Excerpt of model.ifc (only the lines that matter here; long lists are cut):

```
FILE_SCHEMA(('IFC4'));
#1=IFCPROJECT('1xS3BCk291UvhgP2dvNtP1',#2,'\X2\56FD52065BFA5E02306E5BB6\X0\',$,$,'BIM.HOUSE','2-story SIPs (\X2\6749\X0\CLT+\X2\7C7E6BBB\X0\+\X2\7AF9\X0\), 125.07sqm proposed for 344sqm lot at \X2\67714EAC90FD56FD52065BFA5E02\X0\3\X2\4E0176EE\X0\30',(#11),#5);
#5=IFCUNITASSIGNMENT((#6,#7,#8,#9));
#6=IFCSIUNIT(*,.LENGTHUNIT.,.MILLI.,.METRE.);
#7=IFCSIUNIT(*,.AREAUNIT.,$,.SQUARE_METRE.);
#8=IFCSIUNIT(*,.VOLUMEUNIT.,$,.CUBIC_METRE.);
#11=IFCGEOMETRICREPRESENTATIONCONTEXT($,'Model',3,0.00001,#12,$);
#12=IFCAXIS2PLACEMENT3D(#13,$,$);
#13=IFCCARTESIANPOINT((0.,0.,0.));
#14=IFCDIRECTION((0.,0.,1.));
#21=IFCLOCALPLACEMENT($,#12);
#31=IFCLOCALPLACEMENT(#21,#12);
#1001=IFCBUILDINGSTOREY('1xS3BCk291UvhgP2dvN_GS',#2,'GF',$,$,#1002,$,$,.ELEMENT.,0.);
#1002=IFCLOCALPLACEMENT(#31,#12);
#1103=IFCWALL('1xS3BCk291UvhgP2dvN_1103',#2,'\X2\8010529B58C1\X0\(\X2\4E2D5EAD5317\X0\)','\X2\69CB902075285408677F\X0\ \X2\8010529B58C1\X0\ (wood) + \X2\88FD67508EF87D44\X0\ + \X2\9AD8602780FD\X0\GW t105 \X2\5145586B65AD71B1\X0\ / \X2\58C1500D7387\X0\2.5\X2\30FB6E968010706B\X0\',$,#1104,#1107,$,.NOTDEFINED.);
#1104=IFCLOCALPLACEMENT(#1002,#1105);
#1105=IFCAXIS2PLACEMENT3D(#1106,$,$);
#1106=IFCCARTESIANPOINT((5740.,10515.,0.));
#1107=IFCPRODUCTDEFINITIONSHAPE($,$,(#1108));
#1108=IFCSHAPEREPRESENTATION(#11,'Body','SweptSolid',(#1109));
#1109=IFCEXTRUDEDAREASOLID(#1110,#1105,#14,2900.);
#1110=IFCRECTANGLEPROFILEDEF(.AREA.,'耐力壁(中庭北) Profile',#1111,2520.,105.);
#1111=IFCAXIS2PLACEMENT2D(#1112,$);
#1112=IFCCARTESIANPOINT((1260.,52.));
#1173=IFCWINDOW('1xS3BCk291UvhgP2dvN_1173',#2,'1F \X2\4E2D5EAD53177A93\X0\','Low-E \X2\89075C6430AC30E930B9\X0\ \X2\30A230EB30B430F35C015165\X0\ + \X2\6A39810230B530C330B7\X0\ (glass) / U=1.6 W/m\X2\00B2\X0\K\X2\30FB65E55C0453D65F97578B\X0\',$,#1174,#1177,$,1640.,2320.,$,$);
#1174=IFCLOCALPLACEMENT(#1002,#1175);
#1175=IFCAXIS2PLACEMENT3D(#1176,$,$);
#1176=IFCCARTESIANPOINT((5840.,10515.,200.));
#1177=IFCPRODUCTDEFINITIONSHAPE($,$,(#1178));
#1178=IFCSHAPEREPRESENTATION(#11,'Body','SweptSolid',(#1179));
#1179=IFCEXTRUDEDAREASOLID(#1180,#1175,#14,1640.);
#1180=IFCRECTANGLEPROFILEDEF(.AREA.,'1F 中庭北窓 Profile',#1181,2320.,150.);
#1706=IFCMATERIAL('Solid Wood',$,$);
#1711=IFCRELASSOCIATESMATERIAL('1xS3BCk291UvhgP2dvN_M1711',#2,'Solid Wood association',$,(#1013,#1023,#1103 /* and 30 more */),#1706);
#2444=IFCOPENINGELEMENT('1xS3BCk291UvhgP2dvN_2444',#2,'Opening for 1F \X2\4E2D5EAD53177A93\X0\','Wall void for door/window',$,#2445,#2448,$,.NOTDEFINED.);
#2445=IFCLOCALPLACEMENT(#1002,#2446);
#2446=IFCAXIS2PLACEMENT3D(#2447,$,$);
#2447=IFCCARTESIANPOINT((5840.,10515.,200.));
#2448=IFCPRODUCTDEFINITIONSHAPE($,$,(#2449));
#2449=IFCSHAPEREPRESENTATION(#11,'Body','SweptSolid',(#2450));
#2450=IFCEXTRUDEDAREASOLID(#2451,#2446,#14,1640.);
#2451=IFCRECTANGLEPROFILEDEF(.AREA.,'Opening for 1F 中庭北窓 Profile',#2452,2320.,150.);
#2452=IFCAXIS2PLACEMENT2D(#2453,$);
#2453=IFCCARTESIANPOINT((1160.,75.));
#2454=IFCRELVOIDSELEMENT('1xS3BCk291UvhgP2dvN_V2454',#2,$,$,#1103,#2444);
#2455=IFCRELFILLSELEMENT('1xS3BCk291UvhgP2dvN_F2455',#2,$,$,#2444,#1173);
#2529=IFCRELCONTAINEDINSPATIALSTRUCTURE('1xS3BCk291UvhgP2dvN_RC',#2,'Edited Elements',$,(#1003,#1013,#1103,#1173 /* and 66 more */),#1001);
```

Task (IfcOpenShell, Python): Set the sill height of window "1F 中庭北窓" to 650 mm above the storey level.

```python
import numpy as np
import ifcopenshell
import ifcopenshell.api.geometry
import ifcopenshell.geom
import ifcopenshell.util.element
import ifcopenshell.util.placement
import ifcopenshell.util.shape
import ifcopenshell.util.unit

model = ifcopenshell.open("model.ifc")
unit_scale = ifcopenshell.util.unit.calculate_unit_scale(model)

window = model.by_guid("1xS3BCk291UvhgP2dvN_1173")
opening = window.FillsVoids[0].RelatingOpeningElement
storey = ifcopenshell.util.element.get_container(window, ifc_class="IfcBuildingStorey")
level = ifcopenshell.util.placement.get_local_placement(storey.ObjectPlacement)[2, 3]

# The opening's origin need not be at the sill, so measure its lowest point.
shape = ifcopenshell.geom.create_shape(ifcopenshell.geom.settings(), opening)
bottom = ifcopenshell.util.shape.get_shape_bottom_elevation(shape, shape.geometry) / unit_scale
dz = level + 0.65 / unit_scale - bottom

shift = np.array([0.0, 0.0, dz])
# The window is not placed relative to its opening, so move both.
for product in (opening, window):
    matrix = ifcopenshell.util.placement.get_local_placement(product.ObjectPlacement)
    matrix[:3, 3] += shift
    ifcopenshell.api.geometry.edit_object_placement(model, product=product, matrix=matrix, is_si=False)

print(f"moved by {dz * unit_scale:+.3f} m")

model.write("model_updated.ifc")
```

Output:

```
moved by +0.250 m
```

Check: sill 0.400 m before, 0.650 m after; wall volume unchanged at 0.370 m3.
